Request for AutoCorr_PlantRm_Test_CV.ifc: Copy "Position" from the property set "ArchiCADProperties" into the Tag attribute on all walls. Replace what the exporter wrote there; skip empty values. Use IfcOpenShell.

First a look at what the model holds.

```python
import ifcopenshell
import ifcopenshell.util.element

model = ifcopenshell.open("AutoCorr_PlantRm_Test_CV.ifc")
print(model.schema)
walls = model.by_type("IfcWall")
print(len(walls), "walls")
for e in walls[:8]:
    source = ifcopenshell.util.element.get_pset(e, "ArchiCADProperties", "Position")
    target = e.Tag
    print(e.id(), repr(source), repr(target), sep=" | ")
```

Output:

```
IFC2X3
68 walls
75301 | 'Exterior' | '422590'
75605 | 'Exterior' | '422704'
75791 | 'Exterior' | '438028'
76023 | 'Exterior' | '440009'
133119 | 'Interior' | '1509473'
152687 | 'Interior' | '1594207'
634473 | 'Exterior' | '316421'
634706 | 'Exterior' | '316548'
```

```python
import ifcopenshell
import ifcopenshell.util.element

model = ifcopenshell.open("AutoCorr_PlantRm_Test_CV.ifc")

count = 0
for e in model.by_type("IfcWall"):
    value = ifcopenshell.util.element.get_pset(e, "ArchiCADProperties", "Position")
    current = e.Tag
    if not value or not value.strip() or current == value:
        continue
    e.Tag = value
    count += 1

print(count, "walls updated")

model.write("AutoCorr_PlantRm_Test_CV_updated.ifc")
```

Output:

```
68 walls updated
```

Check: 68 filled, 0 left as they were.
